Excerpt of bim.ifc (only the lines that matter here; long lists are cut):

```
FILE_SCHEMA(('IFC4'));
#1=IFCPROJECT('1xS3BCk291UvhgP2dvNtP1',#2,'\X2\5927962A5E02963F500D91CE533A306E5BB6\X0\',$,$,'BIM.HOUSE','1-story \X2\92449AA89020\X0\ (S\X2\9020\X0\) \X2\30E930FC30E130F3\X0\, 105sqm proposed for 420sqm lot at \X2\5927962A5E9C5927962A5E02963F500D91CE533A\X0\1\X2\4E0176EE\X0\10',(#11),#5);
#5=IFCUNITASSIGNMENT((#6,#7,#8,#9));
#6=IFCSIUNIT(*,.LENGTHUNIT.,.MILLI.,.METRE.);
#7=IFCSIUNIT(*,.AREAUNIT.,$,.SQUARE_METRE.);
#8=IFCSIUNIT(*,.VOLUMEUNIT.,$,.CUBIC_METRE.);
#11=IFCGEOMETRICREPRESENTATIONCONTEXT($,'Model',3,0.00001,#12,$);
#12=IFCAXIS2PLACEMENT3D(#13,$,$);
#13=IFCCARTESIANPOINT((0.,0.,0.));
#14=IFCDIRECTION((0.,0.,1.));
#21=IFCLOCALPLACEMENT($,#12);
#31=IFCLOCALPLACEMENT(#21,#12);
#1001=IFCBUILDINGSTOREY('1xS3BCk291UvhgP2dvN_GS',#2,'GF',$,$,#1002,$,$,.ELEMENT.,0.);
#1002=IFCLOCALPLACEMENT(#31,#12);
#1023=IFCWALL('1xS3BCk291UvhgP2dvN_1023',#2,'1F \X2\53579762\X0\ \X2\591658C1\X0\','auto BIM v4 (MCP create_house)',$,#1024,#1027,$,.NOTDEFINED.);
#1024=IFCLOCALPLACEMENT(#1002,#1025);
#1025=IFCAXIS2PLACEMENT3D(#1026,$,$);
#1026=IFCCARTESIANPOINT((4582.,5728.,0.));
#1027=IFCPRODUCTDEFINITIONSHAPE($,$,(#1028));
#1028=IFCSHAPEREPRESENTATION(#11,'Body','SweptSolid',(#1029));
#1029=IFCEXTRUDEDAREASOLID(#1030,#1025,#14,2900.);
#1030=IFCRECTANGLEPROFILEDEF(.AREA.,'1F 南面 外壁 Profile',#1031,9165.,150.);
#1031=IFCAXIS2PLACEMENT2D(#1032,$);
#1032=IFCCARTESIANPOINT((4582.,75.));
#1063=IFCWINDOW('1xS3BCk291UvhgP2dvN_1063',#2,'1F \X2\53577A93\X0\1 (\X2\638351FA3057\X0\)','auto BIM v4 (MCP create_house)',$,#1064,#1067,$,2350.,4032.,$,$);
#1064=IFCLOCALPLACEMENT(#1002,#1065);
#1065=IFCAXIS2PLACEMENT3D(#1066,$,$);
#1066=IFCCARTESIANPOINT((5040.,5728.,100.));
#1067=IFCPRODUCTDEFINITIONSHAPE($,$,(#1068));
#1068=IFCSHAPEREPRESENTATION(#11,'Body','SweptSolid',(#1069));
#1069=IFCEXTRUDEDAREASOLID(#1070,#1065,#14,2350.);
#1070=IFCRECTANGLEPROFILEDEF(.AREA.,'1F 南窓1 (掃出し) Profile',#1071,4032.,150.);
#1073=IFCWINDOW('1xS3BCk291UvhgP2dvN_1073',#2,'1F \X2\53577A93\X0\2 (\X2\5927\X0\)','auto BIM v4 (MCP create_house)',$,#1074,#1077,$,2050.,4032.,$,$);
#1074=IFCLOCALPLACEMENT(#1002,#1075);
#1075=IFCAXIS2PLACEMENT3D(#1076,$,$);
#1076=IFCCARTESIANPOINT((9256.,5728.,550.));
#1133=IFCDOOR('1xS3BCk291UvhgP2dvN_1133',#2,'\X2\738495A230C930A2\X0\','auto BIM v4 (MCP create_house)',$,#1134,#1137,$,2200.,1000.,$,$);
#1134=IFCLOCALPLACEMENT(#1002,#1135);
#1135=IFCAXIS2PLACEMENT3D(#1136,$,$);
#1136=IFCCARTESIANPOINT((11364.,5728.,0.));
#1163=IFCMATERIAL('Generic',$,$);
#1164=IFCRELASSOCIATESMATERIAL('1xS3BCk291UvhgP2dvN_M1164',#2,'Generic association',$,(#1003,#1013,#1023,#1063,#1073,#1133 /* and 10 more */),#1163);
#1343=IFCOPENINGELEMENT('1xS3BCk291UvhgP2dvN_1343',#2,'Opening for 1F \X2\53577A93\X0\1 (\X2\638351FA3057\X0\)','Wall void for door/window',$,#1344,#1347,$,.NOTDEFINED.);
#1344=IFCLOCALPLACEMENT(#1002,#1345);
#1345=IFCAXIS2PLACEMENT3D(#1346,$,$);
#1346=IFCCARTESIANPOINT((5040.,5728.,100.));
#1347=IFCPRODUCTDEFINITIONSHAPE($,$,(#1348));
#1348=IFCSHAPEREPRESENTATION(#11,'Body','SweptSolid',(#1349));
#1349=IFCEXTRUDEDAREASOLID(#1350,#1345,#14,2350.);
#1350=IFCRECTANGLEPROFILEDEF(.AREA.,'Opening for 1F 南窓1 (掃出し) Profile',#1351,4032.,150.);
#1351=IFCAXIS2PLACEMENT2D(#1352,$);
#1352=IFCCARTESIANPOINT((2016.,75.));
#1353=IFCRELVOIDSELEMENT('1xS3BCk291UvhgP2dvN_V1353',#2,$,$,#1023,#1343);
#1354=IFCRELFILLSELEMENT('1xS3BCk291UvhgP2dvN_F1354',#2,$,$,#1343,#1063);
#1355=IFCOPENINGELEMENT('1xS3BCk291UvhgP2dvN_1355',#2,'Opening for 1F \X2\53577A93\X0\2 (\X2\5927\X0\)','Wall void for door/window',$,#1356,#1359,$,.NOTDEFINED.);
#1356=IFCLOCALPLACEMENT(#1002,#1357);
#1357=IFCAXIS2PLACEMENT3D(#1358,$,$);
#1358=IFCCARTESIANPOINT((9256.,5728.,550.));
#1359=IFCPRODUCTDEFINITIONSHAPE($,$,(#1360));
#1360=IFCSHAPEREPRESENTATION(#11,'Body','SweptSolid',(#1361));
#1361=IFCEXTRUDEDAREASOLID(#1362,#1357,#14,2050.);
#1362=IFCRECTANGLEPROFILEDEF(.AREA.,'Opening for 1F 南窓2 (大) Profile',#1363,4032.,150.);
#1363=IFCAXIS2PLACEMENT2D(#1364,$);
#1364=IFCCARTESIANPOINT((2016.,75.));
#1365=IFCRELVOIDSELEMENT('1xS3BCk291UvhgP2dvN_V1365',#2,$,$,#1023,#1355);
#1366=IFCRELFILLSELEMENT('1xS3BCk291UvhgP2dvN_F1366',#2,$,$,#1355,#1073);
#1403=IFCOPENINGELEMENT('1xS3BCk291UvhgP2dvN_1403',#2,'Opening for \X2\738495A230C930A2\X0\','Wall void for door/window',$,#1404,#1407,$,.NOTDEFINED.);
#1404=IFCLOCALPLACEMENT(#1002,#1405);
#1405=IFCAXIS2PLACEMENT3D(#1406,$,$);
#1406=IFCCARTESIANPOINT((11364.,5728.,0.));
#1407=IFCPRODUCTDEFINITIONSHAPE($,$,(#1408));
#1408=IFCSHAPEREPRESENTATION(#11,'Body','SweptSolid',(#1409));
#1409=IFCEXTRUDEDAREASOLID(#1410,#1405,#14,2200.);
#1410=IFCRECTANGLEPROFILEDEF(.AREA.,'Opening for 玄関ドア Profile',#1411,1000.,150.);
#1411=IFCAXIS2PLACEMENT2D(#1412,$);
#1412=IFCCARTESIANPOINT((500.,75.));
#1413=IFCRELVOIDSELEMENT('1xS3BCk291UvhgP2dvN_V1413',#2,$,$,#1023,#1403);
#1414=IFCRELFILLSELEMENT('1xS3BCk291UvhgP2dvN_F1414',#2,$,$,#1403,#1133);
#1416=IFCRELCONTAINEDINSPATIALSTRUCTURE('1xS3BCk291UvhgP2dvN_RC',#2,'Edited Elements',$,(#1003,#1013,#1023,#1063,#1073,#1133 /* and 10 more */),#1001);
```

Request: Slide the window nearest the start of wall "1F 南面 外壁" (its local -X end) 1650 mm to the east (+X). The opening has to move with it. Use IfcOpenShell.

```python
import ifcopenshell
import ifcopenshell.api.geometry
import ifcopenshell.util.placement
import ifcopenshell.util.unit

model = ifcopenshell.open("bim.ifc")
unit_scale = ifcopenshell.util.unit.calculate_unit_scale(model)

window = model.by_guid("1xS3BCk291UvhgP2dvN_1063")
opening = window.FillsVoids[0].RelatingOpeningElement
wall = opening.VoidsElements[0].RelatingBuildingElement

wall_matrix = ifcopenshell.util.placement.get_local_placement(wall.ObjectPlacement)
shift = wall_matrix[:3, 0] * 1.65 / unit_scale
before = ifcopenshell.util.placement.get_local_placement(window.ObjectPlacement)[:3, 3].copy()

# The window is not placed relative to its opening, so move both.
for product in (opening, window):
    matrix = ifcopenshell.util.placement.get_local_placement(product.ObjectPlacement)
    matrix[:3, 3] += shift
    ifcopenshell.api.geometry.edit_object_placement(model, product=product, matrix=matrix, is_si=False)

after = ifcopenshell.util.placement.get_local_placement(window.ObjectPlacement)[:3, 3]
print("window moved by", (after - before).round(3) + 0.0)

model.write("bim_edited.ifc")
```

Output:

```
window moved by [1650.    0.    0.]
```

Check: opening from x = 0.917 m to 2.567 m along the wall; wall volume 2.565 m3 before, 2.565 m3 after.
